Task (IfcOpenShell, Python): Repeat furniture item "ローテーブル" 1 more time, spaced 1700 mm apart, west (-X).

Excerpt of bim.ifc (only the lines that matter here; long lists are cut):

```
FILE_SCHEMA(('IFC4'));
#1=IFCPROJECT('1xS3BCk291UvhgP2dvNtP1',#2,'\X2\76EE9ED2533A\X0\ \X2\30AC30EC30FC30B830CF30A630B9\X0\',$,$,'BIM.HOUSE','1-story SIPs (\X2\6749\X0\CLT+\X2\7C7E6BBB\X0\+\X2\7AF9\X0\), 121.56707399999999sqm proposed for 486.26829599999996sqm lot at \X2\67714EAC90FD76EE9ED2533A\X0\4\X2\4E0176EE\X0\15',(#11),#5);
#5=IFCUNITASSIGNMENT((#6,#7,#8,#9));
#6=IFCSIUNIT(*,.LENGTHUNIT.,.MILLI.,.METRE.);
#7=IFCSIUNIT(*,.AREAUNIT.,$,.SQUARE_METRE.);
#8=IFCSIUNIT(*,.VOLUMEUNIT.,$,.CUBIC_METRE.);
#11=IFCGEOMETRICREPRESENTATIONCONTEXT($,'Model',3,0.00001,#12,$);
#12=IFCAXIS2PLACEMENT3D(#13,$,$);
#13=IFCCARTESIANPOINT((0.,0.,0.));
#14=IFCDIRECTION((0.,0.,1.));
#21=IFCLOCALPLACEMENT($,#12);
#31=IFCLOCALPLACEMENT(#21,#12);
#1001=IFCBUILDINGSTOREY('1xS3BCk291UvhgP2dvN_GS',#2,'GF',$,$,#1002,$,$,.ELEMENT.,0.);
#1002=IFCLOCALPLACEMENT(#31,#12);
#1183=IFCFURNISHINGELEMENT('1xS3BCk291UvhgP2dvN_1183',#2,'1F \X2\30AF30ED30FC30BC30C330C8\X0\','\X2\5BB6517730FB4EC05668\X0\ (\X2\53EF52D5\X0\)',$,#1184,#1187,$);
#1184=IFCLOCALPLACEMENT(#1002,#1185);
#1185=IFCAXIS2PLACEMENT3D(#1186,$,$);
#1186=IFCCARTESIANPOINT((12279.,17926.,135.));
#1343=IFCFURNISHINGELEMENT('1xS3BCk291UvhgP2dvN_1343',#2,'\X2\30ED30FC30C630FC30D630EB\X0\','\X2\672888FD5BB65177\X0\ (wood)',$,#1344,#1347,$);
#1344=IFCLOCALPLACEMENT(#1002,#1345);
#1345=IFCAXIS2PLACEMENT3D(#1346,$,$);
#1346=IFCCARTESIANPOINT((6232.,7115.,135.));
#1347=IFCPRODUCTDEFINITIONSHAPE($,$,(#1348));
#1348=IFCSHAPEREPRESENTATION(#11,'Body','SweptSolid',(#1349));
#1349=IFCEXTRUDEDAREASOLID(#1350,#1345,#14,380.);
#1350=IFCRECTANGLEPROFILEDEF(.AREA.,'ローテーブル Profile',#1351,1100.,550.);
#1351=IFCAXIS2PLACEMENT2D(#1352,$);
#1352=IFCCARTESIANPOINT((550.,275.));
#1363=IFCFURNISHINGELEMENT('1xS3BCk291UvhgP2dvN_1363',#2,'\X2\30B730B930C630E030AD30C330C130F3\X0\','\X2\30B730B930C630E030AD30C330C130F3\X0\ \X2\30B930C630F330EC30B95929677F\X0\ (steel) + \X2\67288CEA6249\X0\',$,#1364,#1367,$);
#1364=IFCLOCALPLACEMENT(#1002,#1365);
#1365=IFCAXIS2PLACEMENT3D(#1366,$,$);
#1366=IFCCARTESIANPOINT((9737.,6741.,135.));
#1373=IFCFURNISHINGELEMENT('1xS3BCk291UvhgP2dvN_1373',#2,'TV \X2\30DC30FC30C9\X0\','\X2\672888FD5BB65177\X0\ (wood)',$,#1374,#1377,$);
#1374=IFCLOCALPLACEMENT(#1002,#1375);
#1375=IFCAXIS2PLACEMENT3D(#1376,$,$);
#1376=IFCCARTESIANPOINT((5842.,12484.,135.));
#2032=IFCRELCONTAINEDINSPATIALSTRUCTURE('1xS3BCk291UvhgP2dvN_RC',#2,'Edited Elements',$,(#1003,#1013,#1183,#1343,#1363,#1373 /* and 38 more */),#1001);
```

```python
import numpy as np
import ifcopenshell
import ifcopenshell.api.geometry
import ifcopenshell.api.root
import ifcopenshell.util.element
import ifcopenshell.util.placement
import ifcopenshell.util.unit

model = ifcopenshell.open("bim.ifc")
unit_scale = ifcopenshell.util.unit.calculate_unit_scale(model)


def reuse_history(source, copy):
    """copy_class also copies each property set's owner history, people and application; keep the originals."""
    for rel in copy.IsDefinedBy:
        if rel.is_a("IfcRelDefinesByProperties") and (history := rel.RelatingPropertyDefinition.OwnerHistory):
            rel.RelatingPropertyDefinition.OwnerHistory = source.OwnerHistory
            ifcopenshell.util.element.remove_deep2(model, history)


source = model.by_guid("1xS3BCk291UvhgP2dvN_1343")
base = ifcopenshell.util.placement.get_local_placement(source.ObjectPlacement)
step = np.array([-1.0, 0.0, 0.0]) * 1.7 / unit_scale

for i in range(1, 2):
    copy = ifcopenshell.api.root.copy_class(model, product=source)
    copy.Representation = ifcopenshell.util.element.copy_deep(
        model, source.Representation, exclude=["IfcGeometricRepresentationContext", "IfcRepresentationMap"]
    )
    reuse_history(source, copy)
    matrix = base.copy()
    matrix[:3, 3] += i * step
    print("added at", matrix[:3, 3].round(3) + 0.0)
    ifcopenshell.api.geometry.edit_object_placement(model, product=copy, matrix=matrix, is_si=False)

model.write("bim_edited.ifc")
```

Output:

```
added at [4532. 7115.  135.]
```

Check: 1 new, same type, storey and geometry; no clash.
